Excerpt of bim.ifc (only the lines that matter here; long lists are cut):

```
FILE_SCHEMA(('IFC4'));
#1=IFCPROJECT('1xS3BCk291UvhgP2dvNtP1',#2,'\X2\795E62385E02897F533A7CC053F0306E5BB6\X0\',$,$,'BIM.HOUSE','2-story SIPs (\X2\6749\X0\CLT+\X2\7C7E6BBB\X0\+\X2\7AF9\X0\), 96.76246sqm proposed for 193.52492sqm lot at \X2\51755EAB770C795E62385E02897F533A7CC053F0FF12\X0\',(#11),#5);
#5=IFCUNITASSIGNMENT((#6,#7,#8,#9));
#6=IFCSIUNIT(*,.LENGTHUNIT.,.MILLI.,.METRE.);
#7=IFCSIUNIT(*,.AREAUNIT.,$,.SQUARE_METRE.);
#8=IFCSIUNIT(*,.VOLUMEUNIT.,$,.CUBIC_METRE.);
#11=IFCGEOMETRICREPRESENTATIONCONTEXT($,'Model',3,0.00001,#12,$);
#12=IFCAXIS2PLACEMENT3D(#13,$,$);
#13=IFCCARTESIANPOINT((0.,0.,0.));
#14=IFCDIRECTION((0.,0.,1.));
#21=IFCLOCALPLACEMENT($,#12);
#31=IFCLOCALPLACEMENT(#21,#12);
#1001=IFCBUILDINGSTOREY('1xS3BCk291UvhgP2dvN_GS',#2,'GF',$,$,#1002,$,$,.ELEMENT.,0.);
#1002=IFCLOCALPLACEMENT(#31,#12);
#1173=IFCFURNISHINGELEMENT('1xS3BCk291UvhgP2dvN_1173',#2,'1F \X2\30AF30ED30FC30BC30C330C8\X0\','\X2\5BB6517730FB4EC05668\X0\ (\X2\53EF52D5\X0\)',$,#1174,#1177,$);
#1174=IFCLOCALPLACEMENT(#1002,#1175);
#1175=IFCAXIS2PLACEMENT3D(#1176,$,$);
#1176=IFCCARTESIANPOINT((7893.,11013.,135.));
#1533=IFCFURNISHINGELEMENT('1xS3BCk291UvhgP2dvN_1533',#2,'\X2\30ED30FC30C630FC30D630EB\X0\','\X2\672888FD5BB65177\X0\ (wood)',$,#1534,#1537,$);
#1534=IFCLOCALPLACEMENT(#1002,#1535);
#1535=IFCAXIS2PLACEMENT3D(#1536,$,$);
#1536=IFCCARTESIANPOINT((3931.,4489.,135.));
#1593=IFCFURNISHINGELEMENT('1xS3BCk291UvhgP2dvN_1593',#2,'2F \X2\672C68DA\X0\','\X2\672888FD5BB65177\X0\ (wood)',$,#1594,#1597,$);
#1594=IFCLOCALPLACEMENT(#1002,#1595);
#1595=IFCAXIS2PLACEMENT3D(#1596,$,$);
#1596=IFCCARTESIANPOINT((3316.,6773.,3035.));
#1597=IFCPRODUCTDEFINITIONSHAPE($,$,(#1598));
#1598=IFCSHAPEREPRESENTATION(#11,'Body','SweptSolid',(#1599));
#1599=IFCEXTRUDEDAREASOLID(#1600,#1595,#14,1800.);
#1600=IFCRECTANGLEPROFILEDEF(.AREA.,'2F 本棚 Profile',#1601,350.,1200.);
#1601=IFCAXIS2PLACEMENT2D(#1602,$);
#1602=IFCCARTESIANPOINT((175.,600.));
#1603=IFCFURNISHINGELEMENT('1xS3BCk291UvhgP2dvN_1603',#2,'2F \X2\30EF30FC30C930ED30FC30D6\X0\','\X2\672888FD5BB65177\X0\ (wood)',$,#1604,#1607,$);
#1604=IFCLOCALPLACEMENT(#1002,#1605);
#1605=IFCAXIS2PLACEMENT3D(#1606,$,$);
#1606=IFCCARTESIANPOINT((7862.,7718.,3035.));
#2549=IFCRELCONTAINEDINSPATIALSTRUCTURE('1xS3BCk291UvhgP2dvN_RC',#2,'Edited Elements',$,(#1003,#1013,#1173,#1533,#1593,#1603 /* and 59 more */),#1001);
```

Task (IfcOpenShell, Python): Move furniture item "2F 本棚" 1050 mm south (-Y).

```python
import ifcopenshell
import ifcopenshell.api.geometry
import ifcopenshell.util.placement
import ifcopenshell.util.unit

model = ifcopenshell.open("bim.ifc")
unit_scale = ifcopenshell.util.unit.calculate_unit_scale(model)

item = model.by_guid("1xS3BCk291UvhgP2dvN_1593")
matrix = ifcopenshell.util.placement.get_local_placement(item.ObjectPlacement)
matrix[1, 3] -= 1.05 / unit_scale
ifcopenshell.api.geometry.edit_object_placement(model, product=item, matrix=matrix, is_si=False)

print(ifcopenshell.util.placement.get_local_placement(item.ObjectPlacement).round(3) + 0.0)

model.write("bim_edited.ifc")
```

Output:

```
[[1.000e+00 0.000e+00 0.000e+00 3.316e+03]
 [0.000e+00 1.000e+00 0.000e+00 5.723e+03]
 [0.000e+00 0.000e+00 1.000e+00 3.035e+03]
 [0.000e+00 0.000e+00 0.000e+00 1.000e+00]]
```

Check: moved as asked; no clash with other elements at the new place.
